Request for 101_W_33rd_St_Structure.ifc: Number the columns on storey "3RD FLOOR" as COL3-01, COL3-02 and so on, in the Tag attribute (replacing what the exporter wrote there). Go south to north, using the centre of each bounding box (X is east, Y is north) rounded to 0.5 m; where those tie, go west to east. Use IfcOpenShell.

First a look at what the model holds.

```python
import ifcopenshell
import ifcopenshell.util.element
import ifcopenshell.util.placement

model = ifcopenshell.open("101_W_33rd_St_Structure.ifc")
print(model.schema)
storey = next(s for s in model.by_type("IfcBuildingStorey") if s.Name == "3RD FLOOR")
columns = [e for e in ifcopenshell.util.element.get_decomposition(storey) if e.is_a("IfcColumn")]
for e in sorted(columns, key=lambda e: e.id()):
    origin = ifcopenshell.util.placement.get_local_placement(e.ObjectPlacement)[:3, 3]
    print(e.id(), e.Tag, e.Name, origin.round(2) + 0.0, sep=" | ")
```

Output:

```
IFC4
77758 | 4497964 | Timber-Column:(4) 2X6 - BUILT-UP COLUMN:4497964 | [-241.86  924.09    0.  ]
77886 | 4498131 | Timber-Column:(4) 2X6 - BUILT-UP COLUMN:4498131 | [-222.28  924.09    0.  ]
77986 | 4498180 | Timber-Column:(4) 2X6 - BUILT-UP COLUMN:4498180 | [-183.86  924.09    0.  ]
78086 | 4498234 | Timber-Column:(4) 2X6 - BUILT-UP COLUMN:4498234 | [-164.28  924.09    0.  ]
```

```python
import ifcopenshell
import ifcopenshell.geom
import ifcopenshell.util.element
import ifcopenshell.util.shape

model = ifcopenshell.open("101_W_33rd_St_Structure.ifc")
settings = ifcopenshell.geom.settings()
settings.set("use-world-coords", True)


def centre(element):
    shape = ifcopenshell.geom.create_shape(settings, element)
    return ifcopenshell.util.shape.get_bbox_centroid(shape.geometry)


storey = next(s for s in model.by_type("IfcBuildingStorey") if s.Name == "3RD FLOOR")
columns = [e for e in ifcopenshell.util.element.get_decomposition(storey) if e.is_a("IfcColumn")]

# Insertion points can sit at a corner or the storey origin, so sort by the geometry (in metres).
centres = {e: centre(e) for e in columns}
columns.sort(key=lambda e: (round(centres[e][1] / 0.5), centres[e][0]))

for i, e in enumerate(columns, start=1):
    number = f"COL3-{i:02d}"
    e.Tag = number
    print(e.id(), number)

model.write("101_W_33rd_St_Structure_v2.ifc")
```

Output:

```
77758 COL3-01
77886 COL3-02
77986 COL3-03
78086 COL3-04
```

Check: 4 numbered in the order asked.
